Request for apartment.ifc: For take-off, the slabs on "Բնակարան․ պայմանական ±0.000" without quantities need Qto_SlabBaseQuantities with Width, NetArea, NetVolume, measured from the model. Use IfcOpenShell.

First a look at what the model holds.

```python
import ifcopenshell
import ifcopenshell.util.element
import ifcopenshell.util.unit

model = ifcopenshell.open("apartment.ifc")
print(model.schema)
for unit_type in ("LENGTHUNIT", "AREAUNIT", "VOLUMEUNIT"):
    print(unit_type, ifcopenshell.util.unit.calculate_unit_scale(model, unit_type))
storey = next(s for s in model.by_type("IfcBuildingStorey") if s.Name == "Բնակարան․ պայմանական ±0.000")
slabs = [e for e in ifcopenshell.util.element.get_decomposition(storey) if e.is_a("IfcSlab")]
for e in sorted(slabs, key=lambda e: e.id()):
    print(e.id(), e.is_a(), e.Name, list(ifcopenshell.util.element.get_psets(e, qtos_only=True)), sep=" | ")
```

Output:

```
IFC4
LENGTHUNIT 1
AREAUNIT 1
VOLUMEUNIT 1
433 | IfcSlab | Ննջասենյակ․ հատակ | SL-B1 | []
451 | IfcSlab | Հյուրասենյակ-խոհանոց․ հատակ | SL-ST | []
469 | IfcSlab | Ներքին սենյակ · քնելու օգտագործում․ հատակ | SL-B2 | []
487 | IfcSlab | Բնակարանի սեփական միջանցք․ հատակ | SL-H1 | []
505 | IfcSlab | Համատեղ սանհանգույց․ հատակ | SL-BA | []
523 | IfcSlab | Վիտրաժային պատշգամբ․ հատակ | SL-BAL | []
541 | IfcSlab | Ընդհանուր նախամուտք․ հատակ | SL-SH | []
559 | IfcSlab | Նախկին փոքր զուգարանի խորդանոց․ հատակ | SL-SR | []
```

```python
import ifcopenshell
import ifcopenshell.api.pset
import ifcopenshell.geom
import ifcopenshell.util.element
import ifcopenshell.util.shape
import ifcopenshell.util.unit

model = ifcopenshell.open("apartment.ifc")
unit_scale = ifcopenshell.util.unit.calculate_unit_scale(model)
area_scale = ifcopenshell.util.unit.calculate_unit_scale(model, "AREAUNIT")
volume_scale = ifcopenshell.util.unit.calculate_unit_scale(model, "VOLUMEUNIT")
settings = ifcopenshell.geom.settings()

storey = next(s for s in model.by_type("IfcBuildingStorey") if s.Name == "Բնակարան․ պայմանական ±0.000")
slabs = [e for e in ifcopenshell.util.element.get_decomposition(storey) if e.is_a("IfcSlab")]

for e in sorted(slabs, key=lambda e: e.id()):
    if ifcopenshell.util.element.get_psets(e, qtos_only=True, should_inherit=False):
        continue
    # Geometry comes back in metres, in the element's own axes.
    shape = ifcopenshell.geom.create_shape(settings, e)
    values = {
        "Width": ifcopenshell.util.shape.get_z(shape.geometry) / unit_scale,
        "NetArea": ifcopenshell.util.shape.get_footprint_area(shape.geometry) / area_scale,
        "NetVolume": ifcopenshell.util.shape.get_volume(shape.geometry) / volume_scale,
    }
    qto = ifcopenshell.api.pset.add_qto(model, product=e, name="Qto_SlabBaseQuantities")
    ifcopenshell.api.pset.edit_qto(model, qto=qto, properties=values)
    print(e.id(), {k: round(v, 3) for k, v in values.items()})

model.write("apartment_rev.ifc")
```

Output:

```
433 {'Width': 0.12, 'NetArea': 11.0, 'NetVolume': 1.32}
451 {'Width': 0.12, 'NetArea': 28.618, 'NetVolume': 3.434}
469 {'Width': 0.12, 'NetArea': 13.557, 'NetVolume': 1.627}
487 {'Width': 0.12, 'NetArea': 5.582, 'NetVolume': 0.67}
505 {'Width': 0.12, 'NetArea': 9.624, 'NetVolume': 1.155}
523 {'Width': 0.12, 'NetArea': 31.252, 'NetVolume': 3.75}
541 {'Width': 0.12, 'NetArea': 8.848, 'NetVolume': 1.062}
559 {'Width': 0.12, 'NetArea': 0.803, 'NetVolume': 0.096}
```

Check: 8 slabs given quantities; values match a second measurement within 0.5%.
